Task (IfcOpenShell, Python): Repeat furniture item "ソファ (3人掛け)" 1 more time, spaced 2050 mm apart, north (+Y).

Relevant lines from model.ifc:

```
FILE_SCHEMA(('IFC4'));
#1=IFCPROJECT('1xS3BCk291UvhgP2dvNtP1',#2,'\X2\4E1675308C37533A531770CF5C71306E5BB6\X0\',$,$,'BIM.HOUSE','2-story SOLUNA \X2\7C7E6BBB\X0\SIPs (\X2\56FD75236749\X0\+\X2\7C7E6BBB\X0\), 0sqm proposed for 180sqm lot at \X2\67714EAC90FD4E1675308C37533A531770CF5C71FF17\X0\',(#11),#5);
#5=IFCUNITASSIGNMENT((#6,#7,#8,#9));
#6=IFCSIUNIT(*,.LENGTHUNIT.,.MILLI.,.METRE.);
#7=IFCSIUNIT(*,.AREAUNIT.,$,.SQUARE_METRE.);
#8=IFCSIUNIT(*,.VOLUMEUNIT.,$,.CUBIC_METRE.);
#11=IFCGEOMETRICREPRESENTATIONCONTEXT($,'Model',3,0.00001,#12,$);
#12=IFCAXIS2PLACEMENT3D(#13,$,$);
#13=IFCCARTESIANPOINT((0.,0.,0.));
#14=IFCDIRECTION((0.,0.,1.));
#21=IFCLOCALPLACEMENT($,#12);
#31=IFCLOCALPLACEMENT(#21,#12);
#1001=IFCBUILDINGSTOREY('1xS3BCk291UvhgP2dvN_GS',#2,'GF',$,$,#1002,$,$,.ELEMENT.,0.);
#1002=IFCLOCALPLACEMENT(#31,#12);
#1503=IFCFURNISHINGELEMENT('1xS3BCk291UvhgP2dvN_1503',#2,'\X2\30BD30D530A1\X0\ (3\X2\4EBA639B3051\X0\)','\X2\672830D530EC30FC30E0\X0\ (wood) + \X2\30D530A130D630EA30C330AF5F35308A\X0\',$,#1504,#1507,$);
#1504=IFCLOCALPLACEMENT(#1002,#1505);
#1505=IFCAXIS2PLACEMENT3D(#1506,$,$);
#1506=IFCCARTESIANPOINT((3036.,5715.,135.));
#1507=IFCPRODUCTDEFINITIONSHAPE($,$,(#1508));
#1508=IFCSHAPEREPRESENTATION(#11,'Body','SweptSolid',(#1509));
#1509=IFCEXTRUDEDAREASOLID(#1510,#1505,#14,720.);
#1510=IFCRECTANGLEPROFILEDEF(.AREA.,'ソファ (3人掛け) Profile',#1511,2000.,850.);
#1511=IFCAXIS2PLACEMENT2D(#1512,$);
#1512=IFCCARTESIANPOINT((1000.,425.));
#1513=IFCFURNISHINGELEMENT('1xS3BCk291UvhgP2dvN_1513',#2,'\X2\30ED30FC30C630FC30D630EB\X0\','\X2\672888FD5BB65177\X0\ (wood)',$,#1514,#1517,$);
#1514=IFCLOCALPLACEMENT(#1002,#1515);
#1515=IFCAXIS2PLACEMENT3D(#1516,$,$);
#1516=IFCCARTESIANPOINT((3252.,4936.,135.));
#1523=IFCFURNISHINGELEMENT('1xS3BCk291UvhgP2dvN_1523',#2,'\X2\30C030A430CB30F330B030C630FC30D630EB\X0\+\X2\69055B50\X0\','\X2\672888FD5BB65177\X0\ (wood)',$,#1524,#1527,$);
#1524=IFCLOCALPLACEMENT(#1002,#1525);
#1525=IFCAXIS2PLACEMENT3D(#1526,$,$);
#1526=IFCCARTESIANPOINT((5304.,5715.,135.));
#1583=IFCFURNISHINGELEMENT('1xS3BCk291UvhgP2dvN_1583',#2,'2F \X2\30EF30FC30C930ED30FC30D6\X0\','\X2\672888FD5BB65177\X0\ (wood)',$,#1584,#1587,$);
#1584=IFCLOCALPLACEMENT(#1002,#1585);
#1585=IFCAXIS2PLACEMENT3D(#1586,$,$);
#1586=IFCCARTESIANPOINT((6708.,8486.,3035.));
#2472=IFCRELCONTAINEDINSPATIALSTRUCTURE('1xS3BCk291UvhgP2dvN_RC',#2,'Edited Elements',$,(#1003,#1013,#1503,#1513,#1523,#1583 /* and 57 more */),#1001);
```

```python
import numpy as np
import ifcopenshell
import ifcopenshell.api.geometry
import ifcopenshell.api.root
import ifcopenshell.util.element
import ifcopenshell.util.placement
import ifcopenshell.util.unit

model = ifcopenshell.open("model.ifc")
unit_scale = ifcopenshell.util.unit.calculate_unit_scale(model)


def reuse_history(source, copy):
    """copy_class also copies each property set's owner history, people and application; keep the originals."""
    for rel in copy.IsDefinedBy:
        if rel.is_a("IfcRelDefinesByProperties") and (history := rel.RelatingPropertyDefinition.OwnerHistory):
            rel.RelatingPropertyDefinition.OwnerHistory = source.OwnerHistory
            ifcopenshell.util.element.remove_deep2(model, history)


source = model.by_id(1503)
base = ifcopenshell.util.placement.get_local_placement(source.ObjectPlacement)
step = np.array([0.0, 1.0, 0.0]) * 2.05 / unit_scale

for i in range(1, 2):
    copy = ifcopenshell.api.root.copy_class(model, product=source)
    copy.Representation = ifcopenshell.util.element.copy_deep(
        model, source.Representation, exclude=["IfcGeometricRepresentationContext", "IfcRepresentationMap"]
    )
    reuse_history(source, copy)
    matrix = base.copy()
    matrix[:3, 3] += i * step
    print("added at", matrix[:3, 3].round(3) + 0.0)
    ifcopenshell.api.geometry.edit_object_placement(model, product=copy, matrix=matrix, is_si=False)

model.write("model_v2.ifc")
```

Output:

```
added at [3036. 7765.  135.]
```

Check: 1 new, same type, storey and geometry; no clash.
